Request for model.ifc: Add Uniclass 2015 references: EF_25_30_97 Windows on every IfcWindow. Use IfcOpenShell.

First a look at what the model holds.

```python
import ifcopenshell

model = ifcopenshell.open("model.ifc")
print(model.schema)
print("classifications:", [c.Name for c in model.by_type("IfcClassification")])
for ifc_class in ("IfcDoor", "IfcRoof", "IfcStair", "IfcWall", "IfcWindow"):
    print(ifc_class, len(model.by_type(ifc_class)))
```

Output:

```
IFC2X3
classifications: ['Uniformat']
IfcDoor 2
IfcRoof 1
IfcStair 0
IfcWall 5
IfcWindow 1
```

```python
import ifcopenshell
import ifcopenshell.api.classification

model = ifcopenshell.open("model.ifc")

# IFC2X3 requires Source and Edition and has no link from the project to the system.
system = model.create_entity("IfcClassification", Source="NBS", Edition="2015", Name="Uniclass 2015")

codes = {
    "IfcWindow": ("EF_25_30_97", "Windows"),
}
for ifc_class, (code, name) in codes.items():
    products = model.by_type(ifc_class)
    ifcopenshell.api.classification.add_reference(
        model, products=products, classification=system, identification=code, name=name
    )
    print(code, len(products))

model.write("model_v2.ifc")
```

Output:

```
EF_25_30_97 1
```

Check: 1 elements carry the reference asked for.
